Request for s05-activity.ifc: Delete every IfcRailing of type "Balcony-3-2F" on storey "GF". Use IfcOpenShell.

First a look at what the model holds.

```python
import ifcopenshell
import ifcopenshell.util.element

model = ifcopenshell.open("s05-activity.ifc")
print(model.schema)
storey = next(s for s in model.by_type("IfcBuildingStorey") if s.Name == "GF")
railings = [e for e in ifcopenshell.util.element.get_decomposition(storey) if e.is_a("IfcRailing")]
seen = {}
for e in railings:
    element_type = ifcopenshell.util.element.get_type(e)
    name = element_type.Name if element_type not in (None, e) else None
    seen[name] = seen.get(name, 0) + 1
for name, count in sorted(seen.items(), key=str):
    print(count, "x", name)
```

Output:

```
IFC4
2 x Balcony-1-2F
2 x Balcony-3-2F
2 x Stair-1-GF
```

```python
import ifcopenshell
import ifcopenshell.api.root
import ifcopenshell.util.element

model = ifcopenshell.open("s05-activity.ifc")

storey = next(s for s in model.by_type("IfcBuildingStorey") if s.Name == "GF")
railings = [e for e in ifcopenshell.util.element.get_decomposition(storey) if e.is_a("IfcRailing")]
targets = [e for e in railings if (t := ifcopenshell.util.element.get_type(e)) not in (None, e) and t.Name == "Balcony-3-2F"]

for e in targets:
    ifcopenshell.api.root.remove_product(model, product=e)
print(len(targets), "removed")

model.write("s05-activity_edited.ifc")
```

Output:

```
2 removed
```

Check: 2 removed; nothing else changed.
